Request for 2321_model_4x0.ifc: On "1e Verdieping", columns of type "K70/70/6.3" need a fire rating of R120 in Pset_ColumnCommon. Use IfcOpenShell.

First a look at what the model holds.

```python
import ifcopenshell
import ifcopenshell.util.element

model = ifcopenshell.open("2321_model_4x0.ifc")
print(model.schema)
storey = next(s for s in model.by_type("IfcBuildingStorey") if s.Name == "1e Verdieping")
columns = [e for e in ifcopenshell.util.element.get_decomposition(storey) if e.is_a("IfcColumn")]
seen = {}
for e in columns:
    element_type = ifcopenshell.util.element.get_type(e)
    key = (element_type.Name if element_type != e and element_type else None, ifcopenshell.util.element.get_pset(e, "Pset_ColumnCommon", "FireRating"))
    seen[key] = seen.get(key, 0) + 1
for (name, value), count in sorted(seen.items(), key=str):
    print(count, "x", name, "|", value)
```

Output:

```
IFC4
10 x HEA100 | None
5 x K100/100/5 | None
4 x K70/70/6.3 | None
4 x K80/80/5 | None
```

```python
import ifcopenshell
import ifcopenshell.api.pset
import ifcopenshell.util.element

model = ifcopenshell.open("2321_model_4x0.ifc")

storey = next(s for s in model.by_type("IfcBuildingStorey") if s.Name == "1e Verdieping")
columns = [e for e in ifcopenshell.util.element.get_decomposition(storey) if e.is_a("IfcColumn")]

count = 0
for e in columns:
    element_type = ifcopenshell.util.element.get_type(e)
    if element_type in (None, e) or element_type.Name != "K70/70/6.3":
        continue
    # add_pset returns the element's existing set when there is one.
    pset = ifcopenshell.api.pset.add_pset(model, product=e, name="Pset_ColumnCommon")
    ifcopenshell.api.pset.edit_pset(model, pset=pset, properties={"FireRating": "R120"})
    count += 1

print(count, "columns updated")

model.write("2321_model_4x0_rev.ifc")
```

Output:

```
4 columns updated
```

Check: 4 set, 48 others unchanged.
